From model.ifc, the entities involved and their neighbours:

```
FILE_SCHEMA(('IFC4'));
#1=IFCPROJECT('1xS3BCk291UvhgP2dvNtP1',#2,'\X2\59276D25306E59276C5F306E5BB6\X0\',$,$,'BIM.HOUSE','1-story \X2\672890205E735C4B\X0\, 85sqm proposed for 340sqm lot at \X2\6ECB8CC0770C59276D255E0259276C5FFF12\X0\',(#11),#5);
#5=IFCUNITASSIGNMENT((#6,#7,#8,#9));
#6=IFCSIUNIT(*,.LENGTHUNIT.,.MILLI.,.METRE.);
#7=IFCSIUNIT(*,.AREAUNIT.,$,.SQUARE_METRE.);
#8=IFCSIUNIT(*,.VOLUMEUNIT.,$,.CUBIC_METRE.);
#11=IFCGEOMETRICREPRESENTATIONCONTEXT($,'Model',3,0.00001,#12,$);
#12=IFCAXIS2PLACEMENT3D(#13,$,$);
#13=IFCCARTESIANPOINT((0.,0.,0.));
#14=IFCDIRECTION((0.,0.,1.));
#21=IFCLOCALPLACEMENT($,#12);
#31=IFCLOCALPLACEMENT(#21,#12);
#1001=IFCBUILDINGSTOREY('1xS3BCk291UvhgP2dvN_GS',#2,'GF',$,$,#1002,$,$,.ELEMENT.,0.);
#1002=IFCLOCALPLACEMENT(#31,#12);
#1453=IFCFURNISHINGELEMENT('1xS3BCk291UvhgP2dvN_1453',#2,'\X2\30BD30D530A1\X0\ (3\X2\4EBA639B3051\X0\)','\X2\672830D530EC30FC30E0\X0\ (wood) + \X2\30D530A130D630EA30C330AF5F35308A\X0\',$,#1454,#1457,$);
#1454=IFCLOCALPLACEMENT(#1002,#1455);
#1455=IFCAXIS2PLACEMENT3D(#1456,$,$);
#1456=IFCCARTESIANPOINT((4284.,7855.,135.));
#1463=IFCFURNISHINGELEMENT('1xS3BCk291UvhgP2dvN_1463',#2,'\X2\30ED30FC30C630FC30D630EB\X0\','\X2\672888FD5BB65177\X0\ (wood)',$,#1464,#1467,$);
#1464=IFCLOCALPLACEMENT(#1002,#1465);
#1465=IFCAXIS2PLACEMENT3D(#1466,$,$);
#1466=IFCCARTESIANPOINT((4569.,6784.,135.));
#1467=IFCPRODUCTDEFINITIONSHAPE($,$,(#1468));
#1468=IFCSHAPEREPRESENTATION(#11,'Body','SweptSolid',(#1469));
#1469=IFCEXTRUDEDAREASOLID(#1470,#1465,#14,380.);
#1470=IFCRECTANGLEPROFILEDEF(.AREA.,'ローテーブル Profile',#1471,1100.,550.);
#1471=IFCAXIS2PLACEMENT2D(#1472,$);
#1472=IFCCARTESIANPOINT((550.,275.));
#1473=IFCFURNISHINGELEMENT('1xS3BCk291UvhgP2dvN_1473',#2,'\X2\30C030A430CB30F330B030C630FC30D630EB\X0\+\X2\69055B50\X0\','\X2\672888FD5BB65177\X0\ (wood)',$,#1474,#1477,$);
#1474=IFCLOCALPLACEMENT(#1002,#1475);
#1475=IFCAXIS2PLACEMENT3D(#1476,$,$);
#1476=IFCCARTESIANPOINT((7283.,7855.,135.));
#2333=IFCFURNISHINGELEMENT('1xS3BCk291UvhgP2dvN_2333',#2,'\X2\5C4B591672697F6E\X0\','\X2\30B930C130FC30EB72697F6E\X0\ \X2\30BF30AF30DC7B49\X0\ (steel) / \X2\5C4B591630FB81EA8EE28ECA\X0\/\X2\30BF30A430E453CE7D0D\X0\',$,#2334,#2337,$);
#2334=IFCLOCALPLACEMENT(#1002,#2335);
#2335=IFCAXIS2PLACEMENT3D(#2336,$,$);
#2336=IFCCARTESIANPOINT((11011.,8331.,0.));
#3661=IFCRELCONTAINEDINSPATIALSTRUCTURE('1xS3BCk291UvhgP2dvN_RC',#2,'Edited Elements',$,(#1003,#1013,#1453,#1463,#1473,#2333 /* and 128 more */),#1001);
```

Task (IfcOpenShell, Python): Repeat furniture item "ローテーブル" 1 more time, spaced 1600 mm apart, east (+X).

```python
import numpy as np
import ifcopenshell
import ifcopenshell.api.geometry
import ifcopenshell.api.root
import ifcopenshell.util.element
import ifcopenshell.util.placement
import ifcopenshell.util.unit

model = ifcopenshell.open("model.ifc")
unit_scale = ifcopenshell.util.unit.calculate_unit_scale(model)


def reuse_history(source, copy):
    """copy_class also copies each property set's owner history, people and application; keep the originals."""
    for rel in copy.IsDefinedBy:
        if rel.is_a("IfcRelDefinesByProperties") and (history := rel.RelatingPropertyDefinition.OwnerHistory):
            rel.RelatingPropertyDefinition.OwnerHistory = source.OwnerHistory
            ifcopenshell.util.element.remove_deep2(model, history)


source = model.by_guid("1xS3BCk291UvhgP2dvN_1463")
base = ifcopenshell.util.placement.get_local_placement(source.ObjectPlacement)
step = np.array([1.0, 0.0, 0.0]) * 1.6 / unit_scale

for i in range(1, 2):
    copy = ifcopenshell.api.root.copy_class(model, product=source)
    copy.Representation = ifcopenshell.util.element.copy_deep(
        model, source.Representation, exclude=["IfcGeometricRepresentationContext", "IfcRepresentationMap"]
    )
    reuse_history(source, copy)
    matrix = base.copy()
    matrix[:3, 3] += i * step
    print("added at", matrix[:3, 3].round(3) + 0.0)
    ifcopenshell.api.geometry.edit_object_placement(model, product=copy, matrix=matrix, is_si=False)

model.write("model_edited.ifc")
```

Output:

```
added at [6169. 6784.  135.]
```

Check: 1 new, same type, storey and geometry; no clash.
